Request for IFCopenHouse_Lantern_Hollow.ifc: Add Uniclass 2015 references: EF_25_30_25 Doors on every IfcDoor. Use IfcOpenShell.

First a look at what the model holds.

```python
import ifcopenshell

model = ifcopenshell.open("IFCopenHouse_Lantern_Hollow.ifc")
print(model.schema)
print("classifications:", [c.Name for c in model.by_type("IfcClassification")])
for ifc_class in ("IfcDoor", "IfcRoof", "IfcStair", "IfcWall", "IfcWindow"):
    print(ifc_class, len(model.by_type(ifc_class)))
```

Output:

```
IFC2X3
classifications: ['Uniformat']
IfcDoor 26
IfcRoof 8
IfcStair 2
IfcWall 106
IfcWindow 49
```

```python
import ifcopenshell
import ifcopenshell.api.classification

model = ifcopenshell.open("IFCopenHouse_Lantern_Hollow.ifc")

# IFC2X3 requires Source and Edition and has no link from the project to the system.
system = model.create_entity("IfcClassification", Source="NBS", Edition="2015", Name="Uniclass 2015")

codes = {
    "IfcDoor": ("EF_25_30_25", "Doors"),
}
for ifc_class, (code, name) in codes.items():
    products = model.by_type(ifc_class)
    ifcopenshell.api.classification.add_reference(
        model, products=products, classification=system, identification=code, name=name
    )
    print(code, len(products))

model.write("IFCopenHouse_Lantern_Hollow-out.ifc")
```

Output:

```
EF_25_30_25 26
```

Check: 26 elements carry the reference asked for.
